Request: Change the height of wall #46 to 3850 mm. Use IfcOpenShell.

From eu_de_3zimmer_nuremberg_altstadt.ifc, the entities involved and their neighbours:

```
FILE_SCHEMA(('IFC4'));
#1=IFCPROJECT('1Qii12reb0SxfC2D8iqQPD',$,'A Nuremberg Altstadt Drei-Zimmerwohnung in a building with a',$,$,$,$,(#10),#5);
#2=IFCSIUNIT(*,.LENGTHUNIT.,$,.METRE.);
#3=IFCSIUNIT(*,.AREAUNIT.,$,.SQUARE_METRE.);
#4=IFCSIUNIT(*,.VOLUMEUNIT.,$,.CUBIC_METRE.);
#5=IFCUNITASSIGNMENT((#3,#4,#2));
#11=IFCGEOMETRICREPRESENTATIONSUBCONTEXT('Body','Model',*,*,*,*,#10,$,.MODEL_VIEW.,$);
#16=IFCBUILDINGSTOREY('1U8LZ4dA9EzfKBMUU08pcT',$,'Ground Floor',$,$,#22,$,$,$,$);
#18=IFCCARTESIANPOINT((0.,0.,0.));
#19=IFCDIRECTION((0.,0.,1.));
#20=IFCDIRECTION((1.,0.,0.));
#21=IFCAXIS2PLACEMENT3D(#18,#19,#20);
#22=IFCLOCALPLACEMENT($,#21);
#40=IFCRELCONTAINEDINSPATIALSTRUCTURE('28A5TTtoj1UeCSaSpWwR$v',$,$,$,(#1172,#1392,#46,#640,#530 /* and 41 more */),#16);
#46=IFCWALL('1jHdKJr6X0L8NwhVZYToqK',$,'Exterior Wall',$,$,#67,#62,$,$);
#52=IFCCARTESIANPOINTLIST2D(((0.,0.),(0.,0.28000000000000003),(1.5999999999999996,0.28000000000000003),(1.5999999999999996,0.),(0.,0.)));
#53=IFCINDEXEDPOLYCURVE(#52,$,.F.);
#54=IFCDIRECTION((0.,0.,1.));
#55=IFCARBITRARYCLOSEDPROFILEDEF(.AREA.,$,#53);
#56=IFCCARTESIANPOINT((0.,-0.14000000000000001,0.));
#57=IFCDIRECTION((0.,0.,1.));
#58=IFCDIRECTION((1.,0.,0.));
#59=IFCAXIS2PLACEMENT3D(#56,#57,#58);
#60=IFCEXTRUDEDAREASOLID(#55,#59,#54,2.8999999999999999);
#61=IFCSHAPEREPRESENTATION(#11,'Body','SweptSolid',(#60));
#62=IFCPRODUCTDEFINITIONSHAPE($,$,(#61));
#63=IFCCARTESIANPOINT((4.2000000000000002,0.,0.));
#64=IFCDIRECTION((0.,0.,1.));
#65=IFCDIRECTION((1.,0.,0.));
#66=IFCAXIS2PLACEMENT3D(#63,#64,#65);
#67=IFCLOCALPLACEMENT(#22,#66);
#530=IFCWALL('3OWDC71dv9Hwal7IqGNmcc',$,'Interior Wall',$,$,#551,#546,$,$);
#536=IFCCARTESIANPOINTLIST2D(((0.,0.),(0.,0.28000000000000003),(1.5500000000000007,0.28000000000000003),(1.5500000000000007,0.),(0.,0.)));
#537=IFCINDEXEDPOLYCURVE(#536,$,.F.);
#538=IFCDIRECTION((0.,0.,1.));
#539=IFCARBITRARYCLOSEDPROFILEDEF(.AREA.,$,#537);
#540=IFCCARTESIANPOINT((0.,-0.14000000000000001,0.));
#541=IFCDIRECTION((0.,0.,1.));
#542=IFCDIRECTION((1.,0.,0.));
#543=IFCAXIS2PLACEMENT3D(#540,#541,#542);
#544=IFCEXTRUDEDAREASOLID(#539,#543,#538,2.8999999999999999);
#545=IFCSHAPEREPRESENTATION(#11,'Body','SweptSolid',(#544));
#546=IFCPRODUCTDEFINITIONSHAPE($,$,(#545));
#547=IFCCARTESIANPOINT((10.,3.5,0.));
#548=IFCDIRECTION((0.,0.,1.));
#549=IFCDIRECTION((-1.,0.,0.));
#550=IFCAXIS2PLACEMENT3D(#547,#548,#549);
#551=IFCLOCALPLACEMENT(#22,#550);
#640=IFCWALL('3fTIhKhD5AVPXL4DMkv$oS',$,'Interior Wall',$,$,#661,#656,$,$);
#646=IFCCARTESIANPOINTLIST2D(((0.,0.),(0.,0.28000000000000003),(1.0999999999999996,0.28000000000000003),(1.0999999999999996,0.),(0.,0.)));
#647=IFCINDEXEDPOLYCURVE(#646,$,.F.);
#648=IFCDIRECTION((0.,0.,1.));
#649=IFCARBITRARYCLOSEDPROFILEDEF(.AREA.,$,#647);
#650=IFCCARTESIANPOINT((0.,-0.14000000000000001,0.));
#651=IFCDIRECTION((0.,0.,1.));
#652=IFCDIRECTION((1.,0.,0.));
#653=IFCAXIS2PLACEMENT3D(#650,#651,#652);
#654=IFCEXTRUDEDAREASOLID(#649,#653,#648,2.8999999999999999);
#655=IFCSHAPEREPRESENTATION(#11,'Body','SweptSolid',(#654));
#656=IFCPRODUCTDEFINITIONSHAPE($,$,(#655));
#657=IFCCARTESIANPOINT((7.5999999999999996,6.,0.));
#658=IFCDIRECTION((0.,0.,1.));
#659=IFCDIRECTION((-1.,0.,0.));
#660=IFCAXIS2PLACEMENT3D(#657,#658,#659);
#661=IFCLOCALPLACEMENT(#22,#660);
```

```python
import ifcopenshell
import ifcopenshell.geom
import ifcopenshell.util.representation
import ifcopenshell.util.shape

model = ifcopenshell.open("eu_de_3zimmer_nuremberg_altstadt.ifc")
settings = ifcopenshell.geom.settings()


def volume(element):
    """Net volume in cubic metres, openings subtracted."""
    shape = ifcopenshell.geom.create_shape(settings, element)
    return ifcopenshell.util.shape.get_volume(shape.geometry)


wall = model.by_guid("1jHdKJr6X0L8NwhVZYToqK")
before = volume(wall)

body = ifcopenshell.util.representation.get_representation(wall, "Model", "Body")
solid = body.Items[0]
old_height = solid.Depth
solid.Depth = 3.85
after = volume(wall)

print(f"height {old_height:g} -> {solid.Depth:g}, volume {before:.3f} -> {after:.3f} m3")

model.write("eu_de_3zimmer_nuremberg_altstadt_updated.ifc")
```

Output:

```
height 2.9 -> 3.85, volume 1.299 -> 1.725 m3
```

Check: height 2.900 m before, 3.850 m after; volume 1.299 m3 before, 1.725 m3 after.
